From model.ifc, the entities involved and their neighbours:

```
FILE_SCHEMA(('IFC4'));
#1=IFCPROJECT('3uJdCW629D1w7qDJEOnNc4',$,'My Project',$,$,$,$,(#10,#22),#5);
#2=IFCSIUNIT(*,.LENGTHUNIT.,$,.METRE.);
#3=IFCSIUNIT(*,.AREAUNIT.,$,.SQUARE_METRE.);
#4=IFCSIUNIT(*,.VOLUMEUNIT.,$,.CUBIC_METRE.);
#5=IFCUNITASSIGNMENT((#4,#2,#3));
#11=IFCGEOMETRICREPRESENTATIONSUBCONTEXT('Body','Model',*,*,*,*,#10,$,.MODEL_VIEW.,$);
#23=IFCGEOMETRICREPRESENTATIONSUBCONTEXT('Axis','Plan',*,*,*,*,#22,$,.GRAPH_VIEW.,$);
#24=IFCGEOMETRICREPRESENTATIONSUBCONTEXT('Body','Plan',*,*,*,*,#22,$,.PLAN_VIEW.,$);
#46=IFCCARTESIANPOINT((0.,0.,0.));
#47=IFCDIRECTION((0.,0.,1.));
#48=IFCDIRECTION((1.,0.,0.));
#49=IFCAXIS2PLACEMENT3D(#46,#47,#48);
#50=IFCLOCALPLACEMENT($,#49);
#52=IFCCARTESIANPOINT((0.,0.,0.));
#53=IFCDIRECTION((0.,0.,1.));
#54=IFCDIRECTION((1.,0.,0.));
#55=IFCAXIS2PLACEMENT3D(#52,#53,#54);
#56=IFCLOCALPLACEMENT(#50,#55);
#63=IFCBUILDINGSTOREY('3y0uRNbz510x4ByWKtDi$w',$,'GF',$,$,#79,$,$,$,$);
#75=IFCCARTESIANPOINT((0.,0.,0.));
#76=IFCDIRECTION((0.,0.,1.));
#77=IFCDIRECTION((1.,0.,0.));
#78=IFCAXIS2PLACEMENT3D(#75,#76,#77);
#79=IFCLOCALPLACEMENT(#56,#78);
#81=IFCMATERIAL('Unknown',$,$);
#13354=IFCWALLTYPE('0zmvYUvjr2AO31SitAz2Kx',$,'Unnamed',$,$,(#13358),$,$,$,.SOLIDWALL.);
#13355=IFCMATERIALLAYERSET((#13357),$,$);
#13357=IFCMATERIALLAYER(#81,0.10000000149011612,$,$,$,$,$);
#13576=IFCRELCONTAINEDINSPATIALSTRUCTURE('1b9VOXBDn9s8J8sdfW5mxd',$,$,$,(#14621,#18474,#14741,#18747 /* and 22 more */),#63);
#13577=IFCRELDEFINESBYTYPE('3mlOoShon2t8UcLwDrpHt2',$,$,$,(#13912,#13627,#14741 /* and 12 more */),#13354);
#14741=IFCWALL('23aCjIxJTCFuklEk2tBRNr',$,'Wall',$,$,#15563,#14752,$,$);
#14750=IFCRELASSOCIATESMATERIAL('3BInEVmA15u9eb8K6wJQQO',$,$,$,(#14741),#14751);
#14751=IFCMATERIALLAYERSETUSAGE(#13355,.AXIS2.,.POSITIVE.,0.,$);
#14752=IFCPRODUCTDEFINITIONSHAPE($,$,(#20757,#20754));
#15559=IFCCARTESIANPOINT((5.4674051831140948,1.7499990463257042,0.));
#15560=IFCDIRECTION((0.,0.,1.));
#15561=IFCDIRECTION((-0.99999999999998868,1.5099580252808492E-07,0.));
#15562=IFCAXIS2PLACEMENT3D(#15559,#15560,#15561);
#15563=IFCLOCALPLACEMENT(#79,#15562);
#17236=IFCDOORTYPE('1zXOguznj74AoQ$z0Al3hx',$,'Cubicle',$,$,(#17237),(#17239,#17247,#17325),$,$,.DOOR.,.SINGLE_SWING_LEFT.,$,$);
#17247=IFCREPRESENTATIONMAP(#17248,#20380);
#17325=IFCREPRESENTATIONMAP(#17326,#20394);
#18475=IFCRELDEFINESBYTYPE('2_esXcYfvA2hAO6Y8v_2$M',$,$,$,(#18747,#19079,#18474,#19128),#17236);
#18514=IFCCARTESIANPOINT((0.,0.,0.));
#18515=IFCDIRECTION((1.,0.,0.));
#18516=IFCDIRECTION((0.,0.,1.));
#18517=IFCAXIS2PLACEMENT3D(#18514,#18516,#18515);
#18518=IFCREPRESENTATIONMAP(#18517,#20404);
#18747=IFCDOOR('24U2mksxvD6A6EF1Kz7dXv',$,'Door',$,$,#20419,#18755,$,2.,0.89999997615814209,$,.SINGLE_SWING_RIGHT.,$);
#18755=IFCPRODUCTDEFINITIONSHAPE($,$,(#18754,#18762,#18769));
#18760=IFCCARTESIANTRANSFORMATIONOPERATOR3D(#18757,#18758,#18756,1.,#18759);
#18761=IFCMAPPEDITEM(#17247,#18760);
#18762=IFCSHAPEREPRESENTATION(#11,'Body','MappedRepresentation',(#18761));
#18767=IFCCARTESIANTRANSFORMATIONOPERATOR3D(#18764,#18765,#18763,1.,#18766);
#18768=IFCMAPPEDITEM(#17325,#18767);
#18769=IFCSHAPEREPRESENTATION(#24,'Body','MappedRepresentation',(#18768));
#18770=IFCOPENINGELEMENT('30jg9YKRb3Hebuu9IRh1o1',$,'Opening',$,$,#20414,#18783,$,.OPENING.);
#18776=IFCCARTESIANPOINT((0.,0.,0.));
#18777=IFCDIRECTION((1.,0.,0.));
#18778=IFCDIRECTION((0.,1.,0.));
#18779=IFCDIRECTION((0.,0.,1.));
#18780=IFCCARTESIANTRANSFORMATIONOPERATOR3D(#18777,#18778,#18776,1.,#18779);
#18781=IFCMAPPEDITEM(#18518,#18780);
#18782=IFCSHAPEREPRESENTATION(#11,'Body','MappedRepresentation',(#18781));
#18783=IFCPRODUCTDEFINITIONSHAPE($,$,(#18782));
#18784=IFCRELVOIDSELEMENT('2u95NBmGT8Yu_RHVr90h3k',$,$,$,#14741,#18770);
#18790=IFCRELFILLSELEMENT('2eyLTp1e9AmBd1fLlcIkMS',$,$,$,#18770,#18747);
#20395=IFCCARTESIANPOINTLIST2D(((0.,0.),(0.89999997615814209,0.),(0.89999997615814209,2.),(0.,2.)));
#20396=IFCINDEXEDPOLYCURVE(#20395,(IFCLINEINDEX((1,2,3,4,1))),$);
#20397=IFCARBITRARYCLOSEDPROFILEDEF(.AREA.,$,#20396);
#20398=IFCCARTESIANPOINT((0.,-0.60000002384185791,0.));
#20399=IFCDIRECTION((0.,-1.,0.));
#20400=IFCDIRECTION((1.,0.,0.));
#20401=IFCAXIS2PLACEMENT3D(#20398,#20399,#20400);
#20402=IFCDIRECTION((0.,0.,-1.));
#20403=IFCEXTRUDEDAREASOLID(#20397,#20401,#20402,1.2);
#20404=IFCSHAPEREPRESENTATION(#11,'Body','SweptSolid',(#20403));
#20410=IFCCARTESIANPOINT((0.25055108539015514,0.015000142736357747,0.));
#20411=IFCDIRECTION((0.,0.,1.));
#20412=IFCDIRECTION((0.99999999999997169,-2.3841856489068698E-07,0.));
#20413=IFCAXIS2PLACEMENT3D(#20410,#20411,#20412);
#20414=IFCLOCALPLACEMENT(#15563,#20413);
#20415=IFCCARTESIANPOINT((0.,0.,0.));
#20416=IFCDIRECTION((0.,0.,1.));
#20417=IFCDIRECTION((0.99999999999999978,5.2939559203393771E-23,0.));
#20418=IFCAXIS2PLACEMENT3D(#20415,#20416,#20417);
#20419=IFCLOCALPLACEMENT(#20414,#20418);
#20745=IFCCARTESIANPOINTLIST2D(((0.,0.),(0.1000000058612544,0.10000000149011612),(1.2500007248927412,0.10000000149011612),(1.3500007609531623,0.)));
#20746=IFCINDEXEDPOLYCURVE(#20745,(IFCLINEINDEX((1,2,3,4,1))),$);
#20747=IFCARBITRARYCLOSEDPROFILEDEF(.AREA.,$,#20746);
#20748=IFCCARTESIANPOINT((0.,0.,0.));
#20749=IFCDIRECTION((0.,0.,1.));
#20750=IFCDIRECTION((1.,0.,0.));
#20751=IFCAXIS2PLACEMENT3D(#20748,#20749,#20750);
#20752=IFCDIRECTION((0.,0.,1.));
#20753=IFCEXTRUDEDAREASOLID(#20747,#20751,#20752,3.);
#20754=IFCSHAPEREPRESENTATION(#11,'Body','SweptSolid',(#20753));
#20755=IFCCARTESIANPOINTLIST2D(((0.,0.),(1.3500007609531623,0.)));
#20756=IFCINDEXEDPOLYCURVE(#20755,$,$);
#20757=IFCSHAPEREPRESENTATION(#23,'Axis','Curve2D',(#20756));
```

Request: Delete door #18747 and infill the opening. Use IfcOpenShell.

```python
import ifcopenshell
import ifcopenshell.api.feature
import ifcopenshell.api.root
import ifcopenshell.geom
import ifcopenshell.util.shape

model = ifcopenshell.open("model.ifc")
settings = ifcopenshell.geom.settings()


def volume(element):
    """Net volume in cubic metres, openings subtracted."""
    shape = ifcopenshell.geom.create_shape(settings, element)
    return ifcopenshell.util.shape.get_volume(shape.geometry)


door = model.by_id(18747)
opening = door.FillsVoids[0].RelatingOpeningElement
wall = opening.VoidsElements[0].RelatingBuildingElement
before = volume(wall)

ifcopenshell.api.root.remove_product(model, product=door)
ifcopenshell.api.feature.remove_feature(model, feature=opening)

after = volume(wall)

print(f"wall volume {before:.3f} -> {after:.3f} m3")

model.write("model_v2.ifc")
```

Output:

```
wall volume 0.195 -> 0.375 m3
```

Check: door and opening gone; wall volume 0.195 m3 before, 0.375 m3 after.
